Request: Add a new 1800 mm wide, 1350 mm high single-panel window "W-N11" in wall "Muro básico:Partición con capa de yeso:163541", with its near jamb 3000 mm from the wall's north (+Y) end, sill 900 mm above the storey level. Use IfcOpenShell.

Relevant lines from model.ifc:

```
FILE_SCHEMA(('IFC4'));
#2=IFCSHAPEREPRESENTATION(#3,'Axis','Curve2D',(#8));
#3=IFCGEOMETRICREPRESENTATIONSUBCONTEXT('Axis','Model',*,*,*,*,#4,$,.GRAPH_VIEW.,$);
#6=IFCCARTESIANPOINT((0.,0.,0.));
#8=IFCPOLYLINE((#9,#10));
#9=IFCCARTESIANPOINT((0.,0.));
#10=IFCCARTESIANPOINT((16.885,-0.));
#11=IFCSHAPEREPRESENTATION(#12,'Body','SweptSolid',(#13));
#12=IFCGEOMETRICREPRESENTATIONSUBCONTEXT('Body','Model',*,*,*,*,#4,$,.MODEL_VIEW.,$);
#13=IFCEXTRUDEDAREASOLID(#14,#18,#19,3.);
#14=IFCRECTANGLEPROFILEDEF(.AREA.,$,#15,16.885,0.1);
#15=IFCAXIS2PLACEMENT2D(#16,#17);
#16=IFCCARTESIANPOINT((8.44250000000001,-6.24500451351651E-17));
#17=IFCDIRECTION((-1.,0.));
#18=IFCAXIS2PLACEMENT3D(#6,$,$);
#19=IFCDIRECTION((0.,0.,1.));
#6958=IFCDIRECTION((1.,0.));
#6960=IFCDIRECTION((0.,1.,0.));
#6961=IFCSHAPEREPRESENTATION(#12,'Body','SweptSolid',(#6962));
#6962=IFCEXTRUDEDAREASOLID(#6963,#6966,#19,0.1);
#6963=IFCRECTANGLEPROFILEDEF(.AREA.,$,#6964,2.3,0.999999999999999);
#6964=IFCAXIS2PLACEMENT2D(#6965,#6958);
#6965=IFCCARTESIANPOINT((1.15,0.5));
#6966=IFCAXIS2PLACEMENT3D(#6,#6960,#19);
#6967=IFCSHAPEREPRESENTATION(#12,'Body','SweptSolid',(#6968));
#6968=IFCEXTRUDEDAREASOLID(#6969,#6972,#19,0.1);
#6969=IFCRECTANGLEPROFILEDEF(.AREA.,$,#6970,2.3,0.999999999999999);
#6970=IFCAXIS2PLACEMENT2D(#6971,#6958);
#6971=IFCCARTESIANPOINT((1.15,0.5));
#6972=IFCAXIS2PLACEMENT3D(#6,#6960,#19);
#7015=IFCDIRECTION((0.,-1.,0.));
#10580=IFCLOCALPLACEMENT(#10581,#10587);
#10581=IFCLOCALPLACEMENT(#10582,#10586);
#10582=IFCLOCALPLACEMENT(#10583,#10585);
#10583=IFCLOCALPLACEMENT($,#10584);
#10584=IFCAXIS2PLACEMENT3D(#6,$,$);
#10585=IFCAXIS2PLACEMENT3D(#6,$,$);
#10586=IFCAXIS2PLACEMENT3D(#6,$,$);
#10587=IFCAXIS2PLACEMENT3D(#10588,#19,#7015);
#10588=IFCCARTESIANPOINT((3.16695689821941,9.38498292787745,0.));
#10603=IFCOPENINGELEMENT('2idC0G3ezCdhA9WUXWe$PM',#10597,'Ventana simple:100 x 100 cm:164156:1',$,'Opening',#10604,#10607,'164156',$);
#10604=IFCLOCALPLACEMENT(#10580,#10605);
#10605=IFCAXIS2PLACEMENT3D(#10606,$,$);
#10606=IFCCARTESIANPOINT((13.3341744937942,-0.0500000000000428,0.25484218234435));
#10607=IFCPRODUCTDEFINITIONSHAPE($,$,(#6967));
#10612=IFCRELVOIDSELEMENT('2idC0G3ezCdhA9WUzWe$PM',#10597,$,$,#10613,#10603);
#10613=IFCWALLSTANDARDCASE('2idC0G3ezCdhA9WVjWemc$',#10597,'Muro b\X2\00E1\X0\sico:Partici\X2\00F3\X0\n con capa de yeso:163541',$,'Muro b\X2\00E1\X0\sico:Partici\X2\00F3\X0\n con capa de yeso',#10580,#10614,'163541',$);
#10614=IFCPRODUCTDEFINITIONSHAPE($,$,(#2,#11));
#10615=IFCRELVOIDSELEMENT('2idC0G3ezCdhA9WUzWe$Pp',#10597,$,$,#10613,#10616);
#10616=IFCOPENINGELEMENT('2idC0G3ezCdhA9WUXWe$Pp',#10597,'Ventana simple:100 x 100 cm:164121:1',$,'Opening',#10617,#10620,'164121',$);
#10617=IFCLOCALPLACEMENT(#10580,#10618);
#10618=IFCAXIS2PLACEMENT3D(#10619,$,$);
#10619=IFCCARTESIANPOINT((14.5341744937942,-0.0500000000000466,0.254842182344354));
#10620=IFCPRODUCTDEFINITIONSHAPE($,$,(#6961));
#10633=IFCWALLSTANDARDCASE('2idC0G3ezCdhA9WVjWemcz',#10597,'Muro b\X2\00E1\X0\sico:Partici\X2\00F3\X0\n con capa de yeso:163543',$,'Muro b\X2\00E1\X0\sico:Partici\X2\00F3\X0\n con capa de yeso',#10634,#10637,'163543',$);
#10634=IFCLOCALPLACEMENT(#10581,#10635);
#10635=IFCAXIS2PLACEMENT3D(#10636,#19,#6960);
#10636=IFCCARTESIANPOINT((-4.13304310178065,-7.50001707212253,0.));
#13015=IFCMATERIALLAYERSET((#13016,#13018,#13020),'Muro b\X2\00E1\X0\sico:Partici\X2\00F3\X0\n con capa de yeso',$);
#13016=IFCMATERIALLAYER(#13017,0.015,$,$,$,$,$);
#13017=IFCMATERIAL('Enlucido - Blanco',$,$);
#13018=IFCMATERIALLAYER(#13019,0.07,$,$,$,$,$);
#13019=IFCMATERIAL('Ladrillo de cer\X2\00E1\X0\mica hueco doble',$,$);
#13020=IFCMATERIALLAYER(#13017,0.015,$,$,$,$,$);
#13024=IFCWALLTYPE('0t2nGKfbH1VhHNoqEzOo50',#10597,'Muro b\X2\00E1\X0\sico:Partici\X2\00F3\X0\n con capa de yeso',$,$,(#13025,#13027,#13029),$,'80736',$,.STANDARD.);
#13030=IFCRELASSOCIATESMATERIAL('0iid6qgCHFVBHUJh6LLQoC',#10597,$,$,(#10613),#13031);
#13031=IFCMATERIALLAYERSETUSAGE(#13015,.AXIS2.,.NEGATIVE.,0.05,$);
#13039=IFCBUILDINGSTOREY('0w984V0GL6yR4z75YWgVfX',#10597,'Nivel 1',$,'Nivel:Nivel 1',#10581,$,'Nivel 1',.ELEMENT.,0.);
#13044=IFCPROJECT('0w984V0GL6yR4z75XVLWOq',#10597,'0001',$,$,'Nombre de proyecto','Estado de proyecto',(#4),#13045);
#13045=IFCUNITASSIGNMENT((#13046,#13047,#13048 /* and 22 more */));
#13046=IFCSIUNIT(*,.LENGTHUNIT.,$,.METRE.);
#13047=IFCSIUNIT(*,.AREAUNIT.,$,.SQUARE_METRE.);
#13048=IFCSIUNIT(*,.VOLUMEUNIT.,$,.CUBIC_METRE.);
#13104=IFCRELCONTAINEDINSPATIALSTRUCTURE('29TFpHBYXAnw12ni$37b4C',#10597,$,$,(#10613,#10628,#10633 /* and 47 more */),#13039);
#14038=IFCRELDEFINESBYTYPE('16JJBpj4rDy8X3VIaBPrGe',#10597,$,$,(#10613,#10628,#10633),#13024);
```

```python
import numpy as np
import ifcopenshell
import ifcopenshell.api.feature
import ifcopenshell.api.geometry
import ifcopenshell.api.root
import ifcopenshell.api.spatial
import ifcopenshell.geom
import ifcopenshell.util.element
import ifcopenshell.util.placement
import ifcopenshell.util.representation
import ifcopenshell.util.shape
import ifcopenshell.util.unit

model = ifcopenshell.open("model.ifc")
unit_scale = ifcopenshell.util.unit.calculate_unit_scale(model)
settings = ifcopenshell.geom.settings()


def volume(element):
    """Net volume in cubic metres, openings subtracted."""
    shape = ifcopenshell.geom.create_shape(settings, element)
    return ifcopenshell.util.shape.get_volume(shape.geometry)


wall = model.by_guid("2idC0G3ezCdhA9WVjWemc$")
storey = ifcopenshell.util.element.get_container(wall, ifc_class="IfcBuildingStorey")
context = ifcopenshell.util.representation.get_context(model, "Model", "Body", "MODEL_VIEW")
before = volume(wall)

width, height, from_end, sill = 1.8, 1.35, 3, 0.9  # metres

# The wall runs along its own X axis, and the end named is its -X end.
wall_shape = ifcopenshell.geom.create_shape(settings, wall)
x, y, z = ifcopenshell.util.shape.get_vertices(wall_shape.geometry).T
start = x.min() + from_end
face, thickness = float(y.min()), float(y.max() - y.min())
wall_matrix = ifcopenshell.util.placement.get_local_placement(wall.ObjectPlacement)
level = ifcopenshell.util.placement.get_local_placement(storey.ObjectPlacement)[2, 3]


def in_wall(x, y):
    """Placement at x, y metres in the wall's axes, at sill height."""
    matrix = wall_matrix.copy()
    matrix[:, 3] = wall_matrix @ np.array([x / unit_scale, y / unit_scale, 0.0, 1.0])
    matrix[2, 3] = level + sill / unit_scale
    return matrix


# Opening: a box that overshoots both wall faces by 50 mm.
opening = ifcopenshell.api.root.create_entity(model, ifc_class="IfcOpeningElement", predefined_type="OPENING")
box = ifcopenshell.api.geometry.add_wall_representation(
    model, context=context, length=width, height=height, thickness=thickness + 0.1
)
ifcopenshell.api.geometry.assign_representation(model, product=opening, representation=box)
ifcopenshell.api.geometry.edit_object_placement(model, product=opening, matrix=in_wall(start, face - 0.05), is_si=False)
ifcopenshell.api.feature.add_feature(model, feature=opening, element=wall)

window = ifcopenshell.api.root.create_entity(model, ifc_class="IfcWindow", name="W-N11", predefined_type="WINDOW")
window.OverallWidth, window.OverallHeight = width / unit_scale, height / unit_scale
window.PartitioningType = "SINGLE_PANEL"
body = ifcopenshell.api.geometry.add_window_representation(
    model,
    context=context,
    overall_width=window.OverallWidth,
    overall_height=window.OverallHeight,
    partition_type="SINGLE_PANEL",
)
ifcopenshell.api.geometry.assign_representation(model, product=window, representation=body)
ifcopenshell.api.spatial.assign_container(model, products=[window], relating_structure=storey)
ifcopenshell.api.feature.add_filling(model, opening=opening, element=window)

# Centre the window in the wall's thickness.
ifcopenshell.api.geometry.edit_object_placement(model, product=window, matrix=in_wall(start, face), is_si=False)
window_shape = ifcopenshell.geom.create_shape(settings, window)
depth = ifcopenshell.util.shape.get_vertices(window_shape.geometry)[:, 1]
offset = face + thickness / 2 - (depth.min() + depth.max()) / 2
ifcopenshell.api.geometry.edit_object_placement(model, product=window, matrix=in_wall(start, offset), is_si=False)

after = volume(wall)

print(f"wall volume {before:.3f} -> {after:.3f} m3")

model.write("model_updated.ifc")
```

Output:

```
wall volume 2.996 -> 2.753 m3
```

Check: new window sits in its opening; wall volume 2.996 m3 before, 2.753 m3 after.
